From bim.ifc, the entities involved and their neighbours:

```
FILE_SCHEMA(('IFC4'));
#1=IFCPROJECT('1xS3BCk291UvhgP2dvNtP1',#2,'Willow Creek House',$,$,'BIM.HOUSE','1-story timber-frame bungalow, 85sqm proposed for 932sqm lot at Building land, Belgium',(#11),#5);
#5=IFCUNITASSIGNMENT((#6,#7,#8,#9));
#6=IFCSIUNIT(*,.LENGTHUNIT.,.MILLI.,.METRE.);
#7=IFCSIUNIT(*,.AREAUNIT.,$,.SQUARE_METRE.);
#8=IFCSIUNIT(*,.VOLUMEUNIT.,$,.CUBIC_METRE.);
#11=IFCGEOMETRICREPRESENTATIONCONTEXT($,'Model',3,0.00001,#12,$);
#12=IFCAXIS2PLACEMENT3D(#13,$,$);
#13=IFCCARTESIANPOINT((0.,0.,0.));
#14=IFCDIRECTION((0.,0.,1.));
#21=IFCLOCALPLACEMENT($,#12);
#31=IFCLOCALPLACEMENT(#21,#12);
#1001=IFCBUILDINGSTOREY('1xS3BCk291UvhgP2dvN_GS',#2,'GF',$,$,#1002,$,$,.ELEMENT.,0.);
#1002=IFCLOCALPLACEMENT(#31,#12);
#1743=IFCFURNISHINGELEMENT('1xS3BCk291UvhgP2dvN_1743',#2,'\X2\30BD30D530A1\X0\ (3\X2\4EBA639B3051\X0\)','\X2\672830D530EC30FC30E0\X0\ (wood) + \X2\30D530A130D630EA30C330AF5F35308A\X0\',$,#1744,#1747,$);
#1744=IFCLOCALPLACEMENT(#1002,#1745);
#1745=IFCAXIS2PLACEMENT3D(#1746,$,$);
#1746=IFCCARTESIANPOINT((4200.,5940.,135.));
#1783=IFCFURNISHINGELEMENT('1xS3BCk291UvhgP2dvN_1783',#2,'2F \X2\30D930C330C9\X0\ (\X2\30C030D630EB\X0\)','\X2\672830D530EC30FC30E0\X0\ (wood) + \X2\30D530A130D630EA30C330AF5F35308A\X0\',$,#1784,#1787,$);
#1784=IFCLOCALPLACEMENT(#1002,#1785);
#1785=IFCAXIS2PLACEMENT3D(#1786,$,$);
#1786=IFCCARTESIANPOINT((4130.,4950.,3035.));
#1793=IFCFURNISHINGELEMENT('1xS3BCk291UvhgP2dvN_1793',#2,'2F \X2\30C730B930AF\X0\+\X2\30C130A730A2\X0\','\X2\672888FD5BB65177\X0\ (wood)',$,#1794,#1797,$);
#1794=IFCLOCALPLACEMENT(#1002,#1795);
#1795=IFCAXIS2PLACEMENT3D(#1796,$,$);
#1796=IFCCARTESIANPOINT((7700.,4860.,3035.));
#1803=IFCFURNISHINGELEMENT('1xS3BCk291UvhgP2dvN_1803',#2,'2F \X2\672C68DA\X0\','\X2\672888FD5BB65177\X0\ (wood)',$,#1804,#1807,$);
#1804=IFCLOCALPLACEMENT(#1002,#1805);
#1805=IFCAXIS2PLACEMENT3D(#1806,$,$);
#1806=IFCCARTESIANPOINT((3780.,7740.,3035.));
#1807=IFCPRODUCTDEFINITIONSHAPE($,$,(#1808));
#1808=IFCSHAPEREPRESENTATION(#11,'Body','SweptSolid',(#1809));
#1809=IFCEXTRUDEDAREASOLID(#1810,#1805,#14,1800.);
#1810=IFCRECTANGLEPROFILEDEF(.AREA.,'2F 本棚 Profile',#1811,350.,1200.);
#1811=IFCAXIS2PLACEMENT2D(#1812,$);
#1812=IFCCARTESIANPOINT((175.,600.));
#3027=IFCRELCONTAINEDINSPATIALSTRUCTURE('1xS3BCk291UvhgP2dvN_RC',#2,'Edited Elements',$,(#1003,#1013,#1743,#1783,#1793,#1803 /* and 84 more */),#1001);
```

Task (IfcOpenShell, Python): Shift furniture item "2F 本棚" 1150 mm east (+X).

```python
import ifcopenshell
import ifcopenshell.api.geometry
import ifcopenshell.util.placement
import ifcopenshell.util.unit

model = ifcopenshell.open("bim.ifc")
unit_scale = ifcopenshell.util.unit.calculate_unit_scale(model)

item = model.by_guid("1xS3BCk291UvhgP2dvN_1803")
matrix = ifcopenshell.util.placement.get_local_placement(item.ObjectPlacement)
matrix[0, 3] += 1.15 / unit_scale
ifcopenshell.api.geometry.edit_object_placement(model, product=item, matrix=matrix, is_si=False)

print(ifcopenshell.util.placement.get_local_placement(item.ObjectPlacement).round(3) + 0.0)

model.write("bim_v2.ifc")
```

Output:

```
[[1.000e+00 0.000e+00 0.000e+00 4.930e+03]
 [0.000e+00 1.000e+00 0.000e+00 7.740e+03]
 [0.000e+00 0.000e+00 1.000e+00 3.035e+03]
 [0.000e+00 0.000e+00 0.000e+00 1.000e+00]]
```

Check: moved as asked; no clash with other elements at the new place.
